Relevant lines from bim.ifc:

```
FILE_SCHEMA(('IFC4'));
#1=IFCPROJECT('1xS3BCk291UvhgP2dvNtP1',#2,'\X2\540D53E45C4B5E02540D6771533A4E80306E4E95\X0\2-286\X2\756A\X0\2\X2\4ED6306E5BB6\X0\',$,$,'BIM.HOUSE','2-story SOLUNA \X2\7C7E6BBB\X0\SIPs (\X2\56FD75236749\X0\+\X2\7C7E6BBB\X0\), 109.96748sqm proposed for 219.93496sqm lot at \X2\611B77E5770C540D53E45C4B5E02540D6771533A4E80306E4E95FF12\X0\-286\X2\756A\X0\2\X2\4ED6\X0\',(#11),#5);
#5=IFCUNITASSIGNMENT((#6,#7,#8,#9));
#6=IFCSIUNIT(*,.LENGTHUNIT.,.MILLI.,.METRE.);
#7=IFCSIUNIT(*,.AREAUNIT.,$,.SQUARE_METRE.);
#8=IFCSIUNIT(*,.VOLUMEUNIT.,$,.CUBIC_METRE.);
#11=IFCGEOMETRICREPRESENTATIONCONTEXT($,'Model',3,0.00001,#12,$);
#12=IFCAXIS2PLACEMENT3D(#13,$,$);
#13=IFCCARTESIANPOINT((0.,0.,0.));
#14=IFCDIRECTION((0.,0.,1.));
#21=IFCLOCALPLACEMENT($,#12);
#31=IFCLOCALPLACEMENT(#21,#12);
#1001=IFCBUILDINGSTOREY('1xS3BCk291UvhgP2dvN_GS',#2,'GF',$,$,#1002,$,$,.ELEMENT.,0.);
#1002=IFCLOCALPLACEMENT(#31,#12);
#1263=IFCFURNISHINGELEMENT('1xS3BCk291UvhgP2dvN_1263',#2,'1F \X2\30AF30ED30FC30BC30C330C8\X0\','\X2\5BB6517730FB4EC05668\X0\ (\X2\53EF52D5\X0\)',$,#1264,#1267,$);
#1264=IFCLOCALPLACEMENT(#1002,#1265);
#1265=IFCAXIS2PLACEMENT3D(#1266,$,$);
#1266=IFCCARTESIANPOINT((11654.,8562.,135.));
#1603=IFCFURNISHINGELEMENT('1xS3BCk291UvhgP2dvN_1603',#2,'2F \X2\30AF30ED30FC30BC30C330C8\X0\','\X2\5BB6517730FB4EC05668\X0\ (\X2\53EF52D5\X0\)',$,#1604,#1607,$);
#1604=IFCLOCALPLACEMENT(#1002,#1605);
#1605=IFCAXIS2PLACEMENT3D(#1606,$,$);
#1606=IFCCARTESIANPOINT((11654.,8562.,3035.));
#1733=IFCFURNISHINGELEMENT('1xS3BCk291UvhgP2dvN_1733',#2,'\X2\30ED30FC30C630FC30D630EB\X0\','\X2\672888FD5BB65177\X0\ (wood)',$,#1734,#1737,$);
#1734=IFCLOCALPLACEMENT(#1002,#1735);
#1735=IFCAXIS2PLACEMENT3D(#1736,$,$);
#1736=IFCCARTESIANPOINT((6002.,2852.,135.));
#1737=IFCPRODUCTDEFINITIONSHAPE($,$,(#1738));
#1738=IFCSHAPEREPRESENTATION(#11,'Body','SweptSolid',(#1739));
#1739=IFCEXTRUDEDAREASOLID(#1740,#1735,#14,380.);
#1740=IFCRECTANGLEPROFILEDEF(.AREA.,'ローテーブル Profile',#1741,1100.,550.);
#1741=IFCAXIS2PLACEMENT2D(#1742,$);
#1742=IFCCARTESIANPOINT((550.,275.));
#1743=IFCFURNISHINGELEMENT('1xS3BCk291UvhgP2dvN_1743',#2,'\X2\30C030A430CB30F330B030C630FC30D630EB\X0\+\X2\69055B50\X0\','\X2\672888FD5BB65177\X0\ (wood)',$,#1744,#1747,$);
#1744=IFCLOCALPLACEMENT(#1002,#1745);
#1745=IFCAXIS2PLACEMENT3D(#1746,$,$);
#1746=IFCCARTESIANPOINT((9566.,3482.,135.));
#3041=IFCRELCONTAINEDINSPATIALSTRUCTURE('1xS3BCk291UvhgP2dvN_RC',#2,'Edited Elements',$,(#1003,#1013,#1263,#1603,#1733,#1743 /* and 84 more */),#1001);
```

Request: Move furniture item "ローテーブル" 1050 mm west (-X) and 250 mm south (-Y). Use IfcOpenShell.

```python
import ifcopenshell
import ifcopenshell.api.geometry
import ifcopenshell.util.placement

model = ifcopenshell.open("bim.ifc")

item = model.by_guid("1xS3BCk291UvhgP2dvN_1733")
matrix = ifcopenshell.util.placement.get_local_placement(item.ObjectPlacement)
matrix[0, 3] -= 1050.0
matrix[1, 3] -= 250.0
ifcopenshell.api.geometry.edit_object_placement(model, product=item, matrix=matrix, is_si=False)

print(ifcopenshell.util.placement.get_local_placement(item.ObjectPlacement).round(3) + 0.0)

model.write("bim_v2.ifc")
```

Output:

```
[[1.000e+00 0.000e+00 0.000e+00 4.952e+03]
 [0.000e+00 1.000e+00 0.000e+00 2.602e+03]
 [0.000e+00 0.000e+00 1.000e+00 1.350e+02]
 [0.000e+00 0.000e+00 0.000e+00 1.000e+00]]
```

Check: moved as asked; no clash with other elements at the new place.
